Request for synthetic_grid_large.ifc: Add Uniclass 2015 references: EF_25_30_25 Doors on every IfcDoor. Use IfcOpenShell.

First a look at what the model holds.

```python
import ifcopenshell

model = ifcopenshell.open("synthetic_grid_large.ifc")
print(model.schema)
print("classifications:", [c.Name for c in model.by_type("IfcClassification")])
for ifc_class in ("IfcDoor", "IfcRoof", "IfcStair", "IfcWall", "IfcWindow"):
    print(ifc_class, len(model.by_type(ifc_class)))
```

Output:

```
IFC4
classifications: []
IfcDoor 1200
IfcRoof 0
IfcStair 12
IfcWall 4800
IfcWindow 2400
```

```python
import ifcopenshell
import ifcopenshell.api.classification

model = ifcopenshell.open("synthetic_grid_large.ifc")

system = ifcopenshell.api.classification.add_classification(model, classification="Uniclass 2015")

codes = {
    "IfcDoor": ("EF_25_30_25", "Doors"),
}
for ifc_class, (code, name) in codes.items():
    products = model.by_type(ifc_class)
    ifcopenshell.api.classification.add_reference(
        model, products=products, classification=system, identification=code, name=name
    )
    print(code, len(products))

model.write("synthetic_grid_large_v2.ifc")
```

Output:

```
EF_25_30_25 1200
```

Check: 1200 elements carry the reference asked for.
